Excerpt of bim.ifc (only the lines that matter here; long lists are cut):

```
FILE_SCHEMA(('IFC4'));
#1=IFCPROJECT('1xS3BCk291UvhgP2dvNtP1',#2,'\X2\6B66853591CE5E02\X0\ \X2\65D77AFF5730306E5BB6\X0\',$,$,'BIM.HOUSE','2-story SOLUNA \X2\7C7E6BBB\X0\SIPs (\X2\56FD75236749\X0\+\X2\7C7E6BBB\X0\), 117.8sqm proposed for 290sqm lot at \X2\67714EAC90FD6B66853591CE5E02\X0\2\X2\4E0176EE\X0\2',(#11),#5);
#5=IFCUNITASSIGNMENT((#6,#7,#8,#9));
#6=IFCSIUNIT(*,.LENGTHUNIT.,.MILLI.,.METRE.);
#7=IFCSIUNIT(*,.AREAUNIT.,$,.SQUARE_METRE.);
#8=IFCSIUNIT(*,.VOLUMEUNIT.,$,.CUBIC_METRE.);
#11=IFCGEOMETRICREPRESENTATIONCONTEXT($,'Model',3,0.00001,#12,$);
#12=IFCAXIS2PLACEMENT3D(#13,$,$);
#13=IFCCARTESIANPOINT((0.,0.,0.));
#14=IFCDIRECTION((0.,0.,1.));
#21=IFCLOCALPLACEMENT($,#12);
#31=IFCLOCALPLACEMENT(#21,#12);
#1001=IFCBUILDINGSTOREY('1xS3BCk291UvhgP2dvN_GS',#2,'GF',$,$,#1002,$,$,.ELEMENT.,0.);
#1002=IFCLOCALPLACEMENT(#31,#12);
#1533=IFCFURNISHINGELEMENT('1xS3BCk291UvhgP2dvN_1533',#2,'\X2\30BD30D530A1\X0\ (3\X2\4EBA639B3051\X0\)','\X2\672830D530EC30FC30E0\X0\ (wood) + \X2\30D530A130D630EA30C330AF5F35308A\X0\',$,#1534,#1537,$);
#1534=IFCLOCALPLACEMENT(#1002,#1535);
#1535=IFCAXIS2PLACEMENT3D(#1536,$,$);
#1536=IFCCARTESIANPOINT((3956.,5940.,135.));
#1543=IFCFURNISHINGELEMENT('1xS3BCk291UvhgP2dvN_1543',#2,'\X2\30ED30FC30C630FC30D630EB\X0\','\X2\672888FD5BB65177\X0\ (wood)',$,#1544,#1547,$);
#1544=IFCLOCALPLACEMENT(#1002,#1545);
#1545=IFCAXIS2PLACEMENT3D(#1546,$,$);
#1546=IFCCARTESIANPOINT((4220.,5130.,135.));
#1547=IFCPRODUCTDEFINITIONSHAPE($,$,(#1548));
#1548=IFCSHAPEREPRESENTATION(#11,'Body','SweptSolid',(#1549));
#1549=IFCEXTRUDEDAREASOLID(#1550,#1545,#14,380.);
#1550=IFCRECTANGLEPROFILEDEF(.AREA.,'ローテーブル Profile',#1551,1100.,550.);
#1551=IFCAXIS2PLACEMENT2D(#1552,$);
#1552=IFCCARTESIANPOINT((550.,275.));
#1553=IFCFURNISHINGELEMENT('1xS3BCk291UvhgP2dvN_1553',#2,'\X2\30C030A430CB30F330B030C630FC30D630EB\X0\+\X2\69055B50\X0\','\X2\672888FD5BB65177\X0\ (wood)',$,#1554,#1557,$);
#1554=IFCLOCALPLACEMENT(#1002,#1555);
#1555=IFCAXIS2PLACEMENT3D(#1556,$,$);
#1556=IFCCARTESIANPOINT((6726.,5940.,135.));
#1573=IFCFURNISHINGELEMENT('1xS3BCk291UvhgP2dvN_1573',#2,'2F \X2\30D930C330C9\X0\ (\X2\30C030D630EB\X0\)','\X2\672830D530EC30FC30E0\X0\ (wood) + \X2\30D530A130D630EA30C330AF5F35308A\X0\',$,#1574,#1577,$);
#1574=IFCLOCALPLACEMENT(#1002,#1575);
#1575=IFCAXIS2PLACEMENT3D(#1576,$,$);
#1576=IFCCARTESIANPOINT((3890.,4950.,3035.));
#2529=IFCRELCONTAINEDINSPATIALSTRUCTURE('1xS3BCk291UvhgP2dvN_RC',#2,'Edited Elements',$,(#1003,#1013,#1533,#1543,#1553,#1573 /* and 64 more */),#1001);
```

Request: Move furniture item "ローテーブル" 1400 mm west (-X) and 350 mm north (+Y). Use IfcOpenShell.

```python
import ifcopenshell
import ifcopenshell.api.geometry
import ifcopenshell.util.placement
import ifcopenshell.util.unit

model = ifcopenshell.open("bim.ifc")
unit_scale = ifcopenshell.util.unit.calculate_unit_scale(model)

item = model.by_guid("1xS3BCk291UvhgP2dvN_1543")
matrix = ifcopenshell.util.placement.get_local_placement(item.ObjectPlacement)
matrix[0, 3] -= 1.4 / unit_scale
matrix[1, 3] += 0.35 / unit_scale
ifcopenshell.api.geometry.edit_object_placement(model, product=item, matrix=matrix, is_si=False)

print(ifcopenshell.util.placement.get_local_placement(item.ObjectPlacement).round(3) + 0.0)

model.write("bim_v2.ifc")
```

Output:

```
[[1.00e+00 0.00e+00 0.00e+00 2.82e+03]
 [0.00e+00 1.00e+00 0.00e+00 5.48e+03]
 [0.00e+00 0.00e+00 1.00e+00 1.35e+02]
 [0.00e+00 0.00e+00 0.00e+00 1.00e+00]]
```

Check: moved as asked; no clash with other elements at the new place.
